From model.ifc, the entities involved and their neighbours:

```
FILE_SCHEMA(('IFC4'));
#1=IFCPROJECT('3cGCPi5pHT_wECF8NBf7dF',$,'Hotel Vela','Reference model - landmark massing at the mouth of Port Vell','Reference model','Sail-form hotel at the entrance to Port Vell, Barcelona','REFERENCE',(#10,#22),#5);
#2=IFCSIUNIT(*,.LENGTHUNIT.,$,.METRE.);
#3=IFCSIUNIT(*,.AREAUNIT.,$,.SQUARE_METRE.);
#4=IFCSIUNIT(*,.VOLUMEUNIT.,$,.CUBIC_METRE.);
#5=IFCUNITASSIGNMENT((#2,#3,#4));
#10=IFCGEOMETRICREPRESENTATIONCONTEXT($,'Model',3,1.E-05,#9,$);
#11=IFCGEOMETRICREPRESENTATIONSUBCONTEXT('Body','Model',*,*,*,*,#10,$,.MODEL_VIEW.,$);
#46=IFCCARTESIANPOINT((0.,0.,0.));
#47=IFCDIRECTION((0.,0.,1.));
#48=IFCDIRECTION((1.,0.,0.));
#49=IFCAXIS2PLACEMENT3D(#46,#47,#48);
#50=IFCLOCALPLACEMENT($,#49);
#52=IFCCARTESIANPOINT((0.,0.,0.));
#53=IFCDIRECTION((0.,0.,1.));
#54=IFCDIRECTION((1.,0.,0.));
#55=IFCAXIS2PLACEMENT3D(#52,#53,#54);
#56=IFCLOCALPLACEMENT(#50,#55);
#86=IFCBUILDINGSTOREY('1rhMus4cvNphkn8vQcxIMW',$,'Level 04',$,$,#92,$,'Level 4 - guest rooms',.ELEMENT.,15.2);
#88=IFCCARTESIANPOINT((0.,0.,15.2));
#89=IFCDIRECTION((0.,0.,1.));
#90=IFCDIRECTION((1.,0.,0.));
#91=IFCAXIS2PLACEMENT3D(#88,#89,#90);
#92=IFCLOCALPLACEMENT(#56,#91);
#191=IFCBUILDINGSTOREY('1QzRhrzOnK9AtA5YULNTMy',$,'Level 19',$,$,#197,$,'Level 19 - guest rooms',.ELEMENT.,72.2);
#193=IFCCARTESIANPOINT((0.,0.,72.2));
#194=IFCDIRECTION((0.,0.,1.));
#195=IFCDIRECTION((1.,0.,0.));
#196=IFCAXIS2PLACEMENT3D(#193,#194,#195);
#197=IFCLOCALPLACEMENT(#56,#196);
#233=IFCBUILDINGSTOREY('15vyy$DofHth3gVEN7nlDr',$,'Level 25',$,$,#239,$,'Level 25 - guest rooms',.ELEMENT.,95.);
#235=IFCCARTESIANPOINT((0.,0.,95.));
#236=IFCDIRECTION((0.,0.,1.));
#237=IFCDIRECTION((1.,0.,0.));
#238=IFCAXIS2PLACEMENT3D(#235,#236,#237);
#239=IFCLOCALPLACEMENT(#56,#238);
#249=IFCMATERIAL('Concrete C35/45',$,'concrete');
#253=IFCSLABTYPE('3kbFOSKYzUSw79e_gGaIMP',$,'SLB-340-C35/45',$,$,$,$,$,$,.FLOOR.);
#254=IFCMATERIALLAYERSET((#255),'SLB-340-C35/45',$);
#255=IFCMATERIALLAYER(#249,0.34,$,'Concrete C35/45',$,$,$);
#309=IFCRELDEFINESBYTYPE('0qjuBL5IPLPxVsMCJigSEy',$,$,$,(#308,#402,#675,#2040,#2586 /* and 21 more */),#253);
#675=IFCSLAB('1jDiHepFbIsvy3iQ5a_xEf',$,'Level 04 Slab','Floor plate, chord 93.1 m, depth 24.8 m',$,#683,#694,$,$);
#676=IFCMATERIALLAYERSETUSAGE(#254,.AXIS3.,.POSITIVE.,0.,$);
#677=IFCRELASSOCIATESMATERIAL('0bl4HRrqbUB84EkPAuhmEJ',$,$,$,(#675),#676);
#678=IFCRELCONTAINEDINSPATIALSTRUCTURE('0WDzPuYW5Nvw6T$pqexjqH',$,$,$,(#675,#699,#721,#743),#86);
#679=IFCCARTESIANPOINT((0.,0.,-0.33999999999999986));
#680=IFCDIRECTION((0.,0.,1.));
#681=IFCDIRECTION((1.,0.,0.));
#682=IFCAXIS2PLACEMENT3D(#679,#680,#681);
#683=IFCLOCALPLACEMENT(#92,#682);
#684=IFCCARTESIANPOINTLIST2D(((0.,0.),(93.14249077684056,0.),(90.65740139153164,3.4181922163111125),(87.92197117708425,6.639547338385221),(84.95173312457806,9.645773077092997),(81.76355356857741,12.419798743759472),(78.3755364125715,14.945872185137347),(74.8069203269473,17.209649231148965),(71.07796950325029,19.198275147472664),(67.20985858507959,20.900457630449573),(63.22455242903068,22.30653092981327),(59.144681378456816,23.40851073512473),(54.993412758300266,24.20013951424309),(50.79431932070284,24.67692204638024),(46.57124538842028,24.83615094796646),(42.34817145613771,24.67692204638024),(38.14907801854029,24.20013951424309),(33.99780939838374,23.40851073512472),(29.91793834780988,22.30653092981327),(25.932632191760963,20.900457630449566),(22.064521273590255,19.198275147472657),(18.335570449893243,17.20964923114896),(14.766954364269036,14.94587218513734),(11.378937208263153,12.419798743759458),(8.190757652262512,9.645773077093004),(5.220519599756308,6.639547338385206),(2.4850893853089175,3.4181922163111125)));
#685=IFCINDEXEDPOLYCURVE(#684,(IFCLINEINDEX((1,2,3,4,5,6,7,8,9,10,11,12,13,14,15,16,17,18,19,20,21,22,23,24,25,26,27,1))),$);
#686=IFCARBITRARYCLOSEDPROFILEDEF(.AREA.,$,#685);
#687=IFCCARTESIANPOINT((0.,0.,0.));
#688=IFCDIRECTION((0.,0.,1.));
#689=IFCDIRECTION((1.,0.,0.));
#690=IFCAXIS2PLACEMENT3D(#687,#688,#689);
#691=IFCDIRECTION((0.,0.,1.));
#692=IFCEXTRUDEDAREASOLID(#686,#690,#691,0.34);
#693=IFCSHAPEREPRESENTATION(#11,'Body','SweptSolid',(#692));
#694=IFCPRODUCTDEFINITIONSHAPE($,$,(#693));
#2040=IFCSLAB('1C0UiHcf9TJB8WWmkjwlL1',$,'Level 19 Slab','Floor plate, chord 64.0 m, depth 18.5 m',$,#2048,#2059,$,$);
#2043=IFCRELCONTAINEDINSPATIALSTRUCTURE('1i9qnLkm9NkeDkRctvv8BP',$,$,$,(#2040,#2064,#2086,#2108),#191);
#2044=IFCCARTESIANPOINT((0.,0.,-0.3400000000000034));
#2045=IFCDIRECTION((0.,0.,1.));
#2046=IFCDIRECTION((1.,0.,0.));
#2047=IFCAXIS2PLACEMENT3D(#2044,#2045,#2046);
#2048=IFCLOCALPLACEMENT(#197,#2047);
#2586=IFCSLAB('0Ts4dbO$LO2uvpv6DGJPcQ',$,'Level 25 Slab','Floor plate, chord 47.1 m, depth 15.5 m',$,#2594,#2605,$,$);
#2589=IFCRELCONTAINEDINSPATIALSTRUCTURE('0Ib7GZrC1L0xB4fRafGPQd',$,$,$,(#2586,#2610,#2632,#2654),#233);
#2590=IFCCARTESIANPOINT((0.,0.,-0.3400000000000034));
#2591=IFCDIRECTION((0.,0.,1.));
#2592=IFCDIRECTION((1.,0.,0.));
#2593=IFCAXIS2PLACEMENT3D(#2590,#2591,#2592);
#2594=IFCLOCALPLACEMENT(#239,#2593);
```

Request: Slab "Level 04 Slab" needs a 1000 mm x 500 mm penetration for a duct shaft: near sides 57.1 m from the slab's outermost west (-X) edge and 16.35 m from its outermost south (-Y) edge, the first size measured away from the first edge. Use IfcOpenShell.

```python
import numpy as np
import ifcopenshell
import ifcopenshell.api.feature
import ifcopenshell.api.geometry
import ifcopenshell.api.root
import ifcopenshell.geom
import ifcopenshell.util.placement
import ifcopenshell.util.representation
import ifcopenshell.util.shape
import ifcopenshell.util.unit

model = ifcopenshell.open("model.ifc")
unit_scale = ifcopenshell.util.unit.calculate_unit_scale(model)
settings = ifcopenshell.geom.settings()


def volume(element):
    """Net volume in cubic metres, openings subtracted."""
    shape = ifcopenshell.geom.create_shape(settings, element)
    return ifcopenshell.util.shape.get_volume(shape.geometry)


slab = model.by_guid("1jDiHepFbIsvy3iQ5a_xEf")
before = volume(slab)

# Extent in the slab's own axes, in metres. The edges named are its -X and -Y sides.
slab_shape = ifcopenshell.geom.create_shape(settings, slab)
vertices = ifcopenshell.util.shape.get_vertices(slab_shape.geometry)
x_min, y_min, bottom = vertices.min(axis=0)
top = vertices[:, 2].max()

opening = ifcopenshell.api.root.create_entity(model, ifc_class="IfcOpeningElement", name="Duct shaft opening", predefined_type="OPENING")
context = ifcopenshell.util.representation.get_context(model, "Model", "Body", "MODEL_VIEW")
width, depth = 1, 0.5
outline = [(0.0, 0.0), (width, 0.0), (width, depth), (0.0, depth), (0.0, 0.0)]
# Overshoot both faces by 50 mm so the cut is clean.
shape = ifcopenshell.api.geometry.add_slab_representation(
    model, context=context, depth=top - bottom + 0.1, polyline=outline
)
ifcopenshell.api.geometry.assign_representation(model, product=opening, representation=shape)

matrix = ifcopenshell.util.placement.get_local_placement(slab.ObjectPlacement)
matrix[:, 3] = matrix @ np.append(np.array([x_min + 57.1, y_min + 16.35, bottom - 0.05]) / unit_scale, 1.0)
ifcopenshell.api.geometry.edit_object_placement(model, product=opening, matrix=matrix, is_si=False)
ifcopenshell.api.feature.add_feature(model, feature=opening, element=slab)

after = volume(slab)

print(f"slab volume {before:.3f} -> {after:.3f} m3")

model.write("model_rev.ifc")
```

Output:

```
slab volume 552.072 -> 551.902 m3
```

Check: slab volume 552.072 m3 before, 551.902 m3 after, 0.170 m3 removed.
